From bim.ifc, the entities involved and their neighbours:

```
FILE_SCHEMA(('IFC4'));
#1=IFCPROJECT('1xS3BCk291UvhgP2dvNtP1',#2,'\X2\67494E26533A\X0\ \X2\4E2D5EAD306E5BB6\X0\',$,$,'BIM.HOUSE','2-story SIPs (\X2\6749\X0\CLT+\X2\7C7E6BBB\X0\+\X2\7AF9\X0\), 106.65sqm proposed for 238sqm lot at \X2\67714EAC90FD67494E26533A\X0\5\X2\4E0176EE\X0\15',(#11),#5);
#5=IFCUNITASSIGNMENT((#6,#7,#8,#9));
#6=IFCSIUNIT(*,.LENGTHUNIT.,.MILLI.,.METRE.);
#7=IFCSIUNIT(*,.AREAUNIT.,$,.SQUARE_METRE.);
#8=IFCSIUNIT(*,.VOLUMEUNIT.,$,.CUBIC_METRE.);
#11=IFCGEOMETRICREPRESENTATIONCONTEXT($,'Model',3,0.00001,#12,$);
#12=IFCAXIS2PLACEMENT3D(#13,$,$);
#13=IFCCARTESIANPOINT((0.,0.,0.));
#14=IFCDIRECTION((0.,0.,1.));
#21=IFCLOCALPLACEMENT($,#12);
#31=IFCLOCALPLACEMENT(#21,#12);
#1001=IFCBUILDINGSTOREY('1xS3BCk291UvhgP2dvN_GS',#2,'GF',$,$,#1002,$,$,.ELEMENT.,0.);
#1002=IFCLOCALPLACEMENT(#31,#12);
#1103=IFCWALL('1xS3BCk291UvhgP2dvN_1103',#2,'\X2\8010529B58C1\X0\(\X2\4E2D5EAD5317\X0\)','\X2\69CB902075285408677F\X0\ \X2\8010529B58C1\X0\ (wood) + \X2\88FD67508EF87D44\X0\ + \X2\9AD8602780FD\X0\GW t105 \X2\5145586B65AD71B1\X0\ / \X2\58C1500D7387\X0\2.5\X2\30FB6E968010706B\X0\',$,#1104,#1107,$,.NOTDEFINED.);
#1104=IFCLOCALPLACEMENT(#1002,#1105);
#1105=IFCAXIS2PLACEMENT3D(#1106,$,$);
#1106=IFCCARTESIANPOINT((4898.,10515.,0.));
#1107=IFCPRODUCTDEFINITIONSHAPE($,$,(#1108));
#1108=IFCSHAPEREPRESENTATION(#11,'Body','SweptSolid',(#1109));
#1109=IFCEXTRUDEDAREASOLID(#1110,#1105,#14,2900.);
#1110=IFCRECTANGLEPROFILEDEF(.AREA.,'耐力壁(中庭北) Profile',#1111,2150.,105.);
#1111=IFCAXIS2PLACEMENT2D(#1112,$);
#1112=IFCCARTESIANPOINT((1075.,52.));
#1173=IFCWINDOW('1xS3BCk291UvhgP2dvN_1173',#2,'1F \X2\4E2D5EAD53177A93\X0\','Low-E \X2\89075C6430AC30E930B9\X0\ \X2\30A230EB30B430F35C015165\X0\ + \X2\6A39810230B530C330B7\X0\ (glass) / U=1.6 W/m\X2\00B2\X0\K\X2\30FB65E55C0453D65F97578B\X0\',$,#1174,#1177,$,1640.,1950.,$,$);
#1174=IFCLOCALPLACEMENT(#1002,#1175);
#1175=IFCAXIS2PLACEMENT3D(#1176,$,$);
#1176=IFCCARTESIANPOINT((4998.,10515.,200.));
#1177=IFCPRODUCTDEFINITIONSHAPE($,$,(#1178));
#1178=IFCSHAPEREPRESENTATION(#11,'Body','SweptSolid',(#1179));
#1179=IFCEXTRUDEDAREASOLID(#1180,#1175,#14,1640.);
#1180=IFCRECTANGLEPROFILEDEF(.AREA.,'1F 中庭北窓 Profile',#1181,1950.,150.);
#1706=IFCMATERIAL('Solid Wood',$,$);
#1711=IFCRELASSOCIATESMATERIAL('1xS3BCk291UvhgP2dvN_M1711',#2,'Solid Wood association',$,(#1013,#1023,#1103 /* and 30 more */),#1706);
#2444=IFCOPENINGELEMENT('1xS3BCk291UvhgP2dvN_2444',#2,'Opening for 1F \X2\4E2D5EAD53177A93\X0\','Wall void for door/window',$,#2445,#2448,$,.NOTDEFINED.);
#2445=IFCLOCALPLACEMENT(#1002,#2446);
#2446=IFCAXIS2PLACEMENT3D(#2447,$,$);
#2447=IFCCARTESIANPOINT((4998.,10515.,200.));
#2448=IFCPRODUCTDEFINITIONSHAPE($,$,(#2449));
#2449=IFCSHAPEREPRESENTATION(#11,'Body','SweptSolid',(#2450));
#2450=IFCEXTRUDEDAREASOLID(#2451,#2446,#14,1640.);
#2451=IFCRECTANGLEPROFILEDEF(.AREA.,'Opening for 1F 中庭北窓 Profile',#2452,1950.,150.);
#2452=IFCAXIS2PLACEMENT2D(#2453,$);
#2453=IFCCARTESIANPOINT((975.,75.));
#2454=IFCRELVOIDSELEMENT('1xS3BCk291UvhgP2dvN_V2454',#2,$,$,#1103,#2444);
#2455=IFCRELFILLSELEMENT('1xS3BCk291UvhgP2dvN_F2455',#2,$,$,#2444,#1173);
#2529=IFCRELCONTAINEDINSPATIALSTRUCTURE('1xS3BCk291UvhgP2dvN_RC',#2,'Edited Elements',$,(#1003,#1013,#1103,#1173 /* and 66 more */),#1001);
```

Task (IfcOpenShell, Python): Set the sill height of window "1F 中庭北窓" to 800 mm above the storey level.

```python
import numpy as np
import ifcopenshell
import ifcopenshell.api.geometry
import ifcopenshell.geom
import ifcopenshell.util.element
import ifcopenshell.util.placement
import ifcopenshell.util.shape
import ifcopenshell.util.unit

model = ifcopenshell.open("bim.ifc")
unit_scale = ifcopenshell.util.unit.calculate_unit_scale(model)

window = model.by_id(1173)
opening = window.FillsVoids[0].RelatingOpeningElement
storey = ifcopenshell.util.element.get_container(window, ifc_class="IfcBuildingStorey")
level = ifcopenshell.util.placement.get_local_placement(storey.ObjectPlacement)[2, 3]

# The opening's origin need not be at the sill, so measure its lowest point.
shape = ifcopenshell.geom.create_shape(ifcopenshell.geom.settings(), opening)
bottom = ifcopenshell.util.shape.get_shape_bottom_elevation(shape, shape.geometry) / unit_scale
dz = level + 800.0 - bottom

shift = np.array([0.0, 0.0, dz])
# The window is not placed relative to its opening, so move both.
for product in (opening, window):
    matrix = ifcopenshell.util.placement.get_local_placement(product.ObjectPlacement)
    matrix[:3, 3] += shift
    ifcopenshell.api.geometry.edit_object_placement(model, product=product, matrix=matrix, is_si=False)

print(f"moved by {dz * unit_scale:+.3f} m")

model.write("bim_edited.ifc")
```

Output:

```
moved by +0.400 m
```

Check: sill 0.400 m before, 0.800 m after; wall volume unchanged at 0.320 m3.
